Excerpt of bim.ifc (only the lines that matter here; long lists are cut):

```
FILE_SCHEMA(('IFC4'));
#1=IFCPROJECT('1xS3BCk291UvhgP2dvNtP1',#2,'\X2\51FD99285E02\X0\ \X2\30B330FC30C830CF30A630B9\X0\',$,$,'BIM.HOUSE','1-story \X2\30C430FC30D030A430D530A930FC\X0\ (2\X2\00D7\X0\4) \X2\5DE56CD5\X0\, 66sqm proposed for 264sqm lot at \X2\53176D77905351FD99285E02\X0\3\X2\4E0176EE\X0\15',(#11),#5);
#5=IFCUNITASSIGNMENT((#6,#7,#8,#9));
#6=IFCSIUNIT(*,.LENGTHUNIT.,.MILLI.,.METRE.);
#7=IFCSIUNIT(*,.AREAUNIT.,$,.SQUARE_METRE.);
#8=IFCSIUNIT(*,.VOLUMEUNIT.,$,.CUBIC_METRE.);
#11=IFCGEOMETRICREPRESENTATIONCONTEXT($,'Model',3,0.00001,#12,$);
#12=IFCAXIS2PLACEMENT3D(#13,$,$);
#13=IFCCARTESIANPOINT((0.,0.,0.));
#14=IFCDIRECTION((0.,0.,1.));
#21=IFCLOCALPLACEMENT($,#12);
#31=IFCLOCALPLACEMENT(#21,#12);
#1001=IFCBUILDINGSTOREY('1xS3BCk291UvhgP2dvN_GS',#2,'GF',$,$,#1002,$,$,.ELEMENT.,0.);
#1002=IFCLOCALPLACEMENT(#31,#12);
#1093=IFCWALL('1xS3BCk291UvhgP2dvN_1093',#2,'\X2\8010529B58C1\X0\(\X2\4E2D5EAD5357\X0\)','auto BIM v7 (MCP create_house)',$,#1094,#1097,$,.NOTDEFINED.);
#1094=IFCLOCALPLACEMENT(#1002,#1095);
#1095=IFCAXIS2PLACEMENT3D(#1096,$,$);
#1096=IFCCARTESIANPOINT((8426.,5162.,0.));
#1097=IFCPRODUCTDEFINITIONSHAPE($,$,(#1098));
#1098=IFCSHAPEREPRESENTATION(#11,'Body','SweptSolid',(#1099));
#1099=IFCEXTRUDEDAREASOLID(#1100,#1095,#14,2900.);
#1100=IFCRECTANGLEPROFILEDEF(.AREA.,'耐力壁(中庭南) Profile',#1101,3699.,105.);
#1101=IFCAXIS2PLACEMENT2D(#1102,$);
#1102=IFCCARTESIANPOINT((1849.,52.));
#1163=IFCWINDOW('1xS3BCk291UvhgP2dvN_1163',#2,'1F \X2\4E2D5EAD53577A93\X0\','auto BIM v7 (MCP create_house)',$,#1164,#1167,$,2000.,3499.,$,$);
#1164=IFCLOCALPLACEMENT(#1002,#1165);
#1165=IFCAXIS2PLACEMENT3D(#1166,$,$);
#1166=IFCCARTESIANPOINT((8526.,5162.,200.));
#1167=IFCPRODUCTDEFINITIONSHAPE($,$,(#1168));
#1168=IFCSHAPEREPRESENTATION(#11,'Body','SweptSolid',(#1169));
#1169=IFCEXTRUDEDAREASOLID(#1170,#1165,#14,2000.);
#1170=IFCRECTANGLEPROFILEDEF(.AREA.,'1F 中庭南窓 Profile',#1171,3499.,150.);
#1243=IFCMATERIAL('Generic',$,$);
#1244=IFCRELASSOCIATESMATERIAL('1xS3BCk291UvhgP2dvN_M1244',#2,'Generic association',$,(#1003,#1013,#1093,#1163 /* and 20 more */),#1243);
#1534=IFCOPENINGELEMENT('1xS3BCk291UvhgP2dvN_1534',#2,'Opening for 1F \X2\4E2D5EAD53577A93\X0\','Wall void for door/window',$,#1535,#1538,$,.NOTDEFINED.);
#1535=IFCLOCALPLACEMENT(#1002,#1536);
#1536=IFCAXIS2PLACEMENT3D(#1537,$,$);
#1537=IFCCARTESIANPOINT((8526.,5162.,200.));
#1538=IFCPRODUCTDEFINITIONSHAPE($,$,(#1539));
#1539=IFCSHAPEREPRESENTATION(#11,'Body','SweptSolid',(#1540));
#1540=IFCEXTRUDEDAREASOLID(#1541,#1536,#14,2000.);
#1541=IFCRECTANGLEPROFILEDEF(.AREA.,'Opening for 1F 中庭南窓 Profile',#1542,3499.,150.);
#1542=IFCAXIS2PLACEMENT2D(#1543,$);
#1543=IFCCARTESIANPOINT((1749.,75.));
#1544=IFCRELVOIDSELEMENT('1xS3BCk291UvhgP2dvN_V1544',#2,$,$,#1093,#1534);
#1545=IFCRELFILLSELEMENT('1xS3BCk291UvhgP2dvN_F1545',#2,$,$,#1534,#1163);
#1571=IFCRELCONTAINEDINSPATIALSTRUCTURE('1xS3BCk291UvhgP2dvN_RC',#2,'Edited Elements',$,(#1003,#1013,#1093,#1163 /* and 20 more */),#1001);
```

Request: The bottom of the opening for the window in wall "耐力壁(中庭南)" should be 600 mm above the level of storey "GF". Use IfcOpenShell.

```python
import numpy as np
import ifcopenshell
import ifcopenshell.api.geometry
import ifcopenshell.geom
import ifcopenshell.util.element
import ifcopenshell.util.placement
import ifcopenshell.util.shape
import ifcopenshell.util.unit

model = ifcopenshell.open("bim.ifc")
unit_scale = ifcopenshell.util.unit.calculate_unit_scale(model)

window = model.by_guid("1xS3BCk291UvhgP2dvN_1163")
opening = window.FillsVoids[0].RelatingOpeningElement
storey = ifcopenshell.util.element.get_container(window, ifc_class="IfcBuildingStorey")
level = ifcopenshell.util.placement.get_local_placement(storey.ObjectPlacement)[2, 3]

# The opening's origin need not be at the sill, so measure its lowest point.
shape = ifcopenshell.geom.create_shape(ifcopenshell.geom.settings(), opening)
bottom = ifcopenshell.util.shape.get_shape_bottom_elevation(shape, shape.geometry) / unit_scale
dz = level + 600.0 - bottom

shift = np.array([0.0, 0.0, dz])
# The window is not placed relative to its opening, so move both.
for product in (opening, window):
    matrix = ifcopenshell.util.placement.get_local_placement(product.ObjectPlacement)
    matrix[:3, 3] += shift
    ifcopenshell.api.geometry.edit_object_placement(model, product=product, matrix=matrix, is_si=False)

print(f"moved by {dz * unit_scale:+.3f} m")

model.write("bim_rev.ifc")
```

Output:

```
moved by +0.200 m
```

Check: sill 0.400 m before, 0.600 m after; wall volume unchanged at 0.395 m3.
